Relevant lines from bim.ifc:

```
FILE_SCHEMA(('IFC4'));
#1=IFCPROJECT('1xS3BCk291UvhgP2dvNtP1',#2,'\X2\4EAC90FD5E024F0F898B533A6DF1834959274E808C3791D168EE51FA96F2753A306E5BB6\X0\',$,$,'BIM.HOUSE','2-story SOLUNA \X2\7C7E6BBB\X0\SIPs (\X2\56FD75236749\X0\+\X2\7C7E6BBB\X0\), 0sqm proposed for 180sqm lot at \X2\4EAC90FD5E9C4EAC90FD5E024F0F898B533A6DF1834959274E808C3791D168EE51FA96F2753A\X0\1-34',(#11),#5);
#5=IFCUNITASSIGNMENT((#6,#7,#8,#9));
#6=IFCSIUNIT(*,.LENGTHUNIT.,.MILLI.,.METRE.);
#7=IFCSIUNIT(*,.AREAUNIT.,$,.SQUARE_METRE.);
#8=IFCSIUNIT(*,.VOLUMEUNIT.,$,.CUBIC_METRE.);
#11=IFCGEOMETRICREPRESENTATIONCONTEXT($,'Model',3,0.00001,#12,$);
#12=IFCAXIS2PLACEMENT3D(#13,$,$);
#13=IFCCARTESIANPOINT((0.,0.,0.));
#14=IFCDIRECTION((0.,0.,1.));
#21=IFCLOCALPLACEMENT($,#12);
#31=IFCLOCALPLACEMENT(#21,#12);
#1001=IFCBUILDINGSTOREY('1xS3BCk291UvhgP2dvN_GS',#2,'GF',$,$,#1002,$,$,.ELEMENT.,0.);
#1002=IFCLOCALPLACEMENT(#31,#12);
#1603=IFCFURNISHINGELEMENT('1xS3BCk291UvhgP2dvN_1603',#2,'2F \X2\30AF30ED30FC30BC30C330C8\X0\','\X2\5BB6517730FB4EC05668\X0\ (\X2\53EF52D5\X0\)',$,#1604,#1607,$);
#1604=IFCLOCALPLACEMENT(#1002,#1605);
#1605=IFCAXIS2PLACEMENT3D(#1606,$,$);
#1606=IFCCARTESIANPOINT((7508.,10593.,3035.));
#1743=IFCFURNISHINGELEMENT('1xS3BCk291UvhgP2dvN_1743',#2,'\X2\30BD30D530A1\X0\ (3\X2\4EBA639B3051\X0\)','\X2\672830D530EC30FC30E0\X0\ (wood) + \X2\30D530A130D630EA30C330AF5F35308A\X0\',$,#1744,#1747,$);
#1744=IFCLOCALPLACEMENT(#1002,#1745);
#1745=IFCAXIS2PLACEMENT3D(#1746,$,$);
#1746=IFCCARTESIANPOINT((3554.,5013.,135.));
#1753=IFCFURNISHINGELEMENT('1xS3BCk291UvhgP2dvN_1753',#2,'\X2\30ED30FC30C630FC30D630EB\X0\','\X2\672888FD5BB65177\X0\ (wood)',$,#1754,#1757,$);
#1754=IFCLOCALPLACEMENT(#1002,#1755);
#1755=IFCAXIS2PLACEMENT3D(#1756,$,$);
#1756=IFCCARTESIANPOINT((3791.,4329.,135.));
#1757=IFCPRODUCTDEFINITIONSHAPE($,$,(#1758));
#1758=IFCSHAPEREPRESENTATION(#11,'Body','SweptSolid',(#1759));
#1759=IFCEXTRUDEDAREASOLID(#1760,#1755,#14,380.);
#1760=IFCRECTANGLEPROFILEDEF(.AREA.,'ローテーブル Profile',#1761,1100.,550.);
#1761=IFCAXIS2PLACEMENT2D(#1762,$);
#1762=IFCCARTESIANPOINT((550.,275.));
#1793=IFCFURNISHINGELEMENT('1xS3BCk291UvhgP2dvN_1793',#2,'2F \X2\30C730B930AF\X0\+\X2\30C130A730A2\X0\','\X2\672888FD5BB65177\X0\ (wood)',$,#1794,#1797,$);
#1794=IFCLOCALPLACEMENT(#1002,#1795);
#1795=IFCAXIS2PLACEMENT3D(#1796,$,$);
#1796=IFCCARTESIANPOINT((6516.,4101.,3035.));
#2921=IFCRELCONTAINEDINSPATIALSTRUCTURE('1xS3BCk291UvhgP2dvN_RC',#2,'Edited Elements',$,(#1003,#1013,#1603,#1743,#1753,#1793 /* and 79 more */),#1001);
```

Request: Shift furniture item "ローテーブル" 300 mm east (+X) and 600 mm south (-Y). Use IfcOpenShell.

```python
import ifcopenshell
import ifcopenshell.api.geometry
import ifcopenshell.util.placement
import ifcopenshell.util.unit

model = ifcopenshell.open("bim.ifc")
unit_scale = ifcopenshell.util.unit.calculate_unit_scale(model)

item = model.by_id(1753)
matrix = ifcopenshell.util.placement.get_local_placement(item.ObjectPlacement)
matrix[0, 3] += 0.3 / unit_scale
matrix[1, 3] -= 0.6 / unit_scale
ifcopenshell.api.geometry.edit_object_placement(model, product=item, matrix=matrix, is_si=False)

print(ifcopenshell.util.placement.get_local_placement(item.ObjectPlacement).round(3) + 0.0)

model.write("bim_edited.ifc")
```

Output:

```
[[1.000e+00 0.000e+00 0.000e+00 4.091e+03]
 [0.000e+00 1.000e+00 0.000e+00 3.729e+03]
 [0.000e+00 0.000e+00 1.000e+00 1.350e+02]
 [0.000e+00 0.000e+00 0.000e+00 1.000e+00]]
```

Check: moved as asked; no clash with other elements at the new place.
